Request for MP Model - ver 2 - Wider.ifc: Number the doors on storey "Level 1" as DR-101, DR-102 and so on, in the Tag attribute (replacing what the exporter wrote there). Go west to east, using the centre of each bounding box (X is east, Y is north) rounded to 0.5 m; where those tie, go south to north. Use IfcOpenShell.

First a look at what the model holds.

```python
import ifcopenshell
import ifcopenshell.util.element
import ifcopenshell.util.placement

model = ifcopenshell.open("MP Model - ver 2 - Wider.ifc")
print(model.schema)
storey = next(s for s in model.by_type("IfcBuildingStorey") if s.Name == "Level 1")
doors = [e for e in ifcopenshell.util.element.get_decomposition(storey) if e.is_a("IfcDoor")]
for e in sorted(doors, key=lambda e: e.id()):
    origin = ifcopenshell.util.placement.get_local_placement(e.ObjectPlacement)[:3, 3]
    print(e.id(), e.Tag, e.Name, origin.round(2) + 0.0, sep=" | ")
```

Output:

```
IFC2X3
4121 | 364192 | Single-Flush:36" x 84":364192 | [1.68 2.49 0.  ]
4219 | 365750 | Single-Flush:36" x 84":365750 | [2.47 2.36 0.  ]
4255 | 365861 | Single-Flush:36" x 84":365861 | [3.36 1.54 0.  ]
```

```python
import ifcopenshell
import ifcopenshell.geom
import ifcopenshell.util.element
import ifcopenshell.util.shape

model = ifcopenshell.open("MP Model - ver 2 - Wider.ifc")
settings = ifcopenshell.geom.settings()
settings.set("use-world-coords", True)


def centre(element):
    shape = ifcopenshell.geom.create_shape(settings, element)
    return ifcopenshell.util.shape.get_bbox_centroid(shape.geometry)


storey = next(s for s in model.by_type("IfcBuildingStorey") if s.Name == "Level 1")
doors = [e for e in ifcopenshell.util.element.get_decomposition(storey) if e.is_a("IfcDoor")]

# Insertion points can sit at a corner or the storey origin, so sort by the geometry (in metres).
centres = {e: centre(e) for e in doors}
doors.sort(key=lambda e: (round(centres[e][0] / 0.5), centres[e][1]))

for i, e in enumerate(doors, start=1):
    number = f"DR-1{i:02d}"
    e.Tag = number
    print(e.id(), number)

model.write("MP Model - ver 2 - Wider_updated.ifc")
```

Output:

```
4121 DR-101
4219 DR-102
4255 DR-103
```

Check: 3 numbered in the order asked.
